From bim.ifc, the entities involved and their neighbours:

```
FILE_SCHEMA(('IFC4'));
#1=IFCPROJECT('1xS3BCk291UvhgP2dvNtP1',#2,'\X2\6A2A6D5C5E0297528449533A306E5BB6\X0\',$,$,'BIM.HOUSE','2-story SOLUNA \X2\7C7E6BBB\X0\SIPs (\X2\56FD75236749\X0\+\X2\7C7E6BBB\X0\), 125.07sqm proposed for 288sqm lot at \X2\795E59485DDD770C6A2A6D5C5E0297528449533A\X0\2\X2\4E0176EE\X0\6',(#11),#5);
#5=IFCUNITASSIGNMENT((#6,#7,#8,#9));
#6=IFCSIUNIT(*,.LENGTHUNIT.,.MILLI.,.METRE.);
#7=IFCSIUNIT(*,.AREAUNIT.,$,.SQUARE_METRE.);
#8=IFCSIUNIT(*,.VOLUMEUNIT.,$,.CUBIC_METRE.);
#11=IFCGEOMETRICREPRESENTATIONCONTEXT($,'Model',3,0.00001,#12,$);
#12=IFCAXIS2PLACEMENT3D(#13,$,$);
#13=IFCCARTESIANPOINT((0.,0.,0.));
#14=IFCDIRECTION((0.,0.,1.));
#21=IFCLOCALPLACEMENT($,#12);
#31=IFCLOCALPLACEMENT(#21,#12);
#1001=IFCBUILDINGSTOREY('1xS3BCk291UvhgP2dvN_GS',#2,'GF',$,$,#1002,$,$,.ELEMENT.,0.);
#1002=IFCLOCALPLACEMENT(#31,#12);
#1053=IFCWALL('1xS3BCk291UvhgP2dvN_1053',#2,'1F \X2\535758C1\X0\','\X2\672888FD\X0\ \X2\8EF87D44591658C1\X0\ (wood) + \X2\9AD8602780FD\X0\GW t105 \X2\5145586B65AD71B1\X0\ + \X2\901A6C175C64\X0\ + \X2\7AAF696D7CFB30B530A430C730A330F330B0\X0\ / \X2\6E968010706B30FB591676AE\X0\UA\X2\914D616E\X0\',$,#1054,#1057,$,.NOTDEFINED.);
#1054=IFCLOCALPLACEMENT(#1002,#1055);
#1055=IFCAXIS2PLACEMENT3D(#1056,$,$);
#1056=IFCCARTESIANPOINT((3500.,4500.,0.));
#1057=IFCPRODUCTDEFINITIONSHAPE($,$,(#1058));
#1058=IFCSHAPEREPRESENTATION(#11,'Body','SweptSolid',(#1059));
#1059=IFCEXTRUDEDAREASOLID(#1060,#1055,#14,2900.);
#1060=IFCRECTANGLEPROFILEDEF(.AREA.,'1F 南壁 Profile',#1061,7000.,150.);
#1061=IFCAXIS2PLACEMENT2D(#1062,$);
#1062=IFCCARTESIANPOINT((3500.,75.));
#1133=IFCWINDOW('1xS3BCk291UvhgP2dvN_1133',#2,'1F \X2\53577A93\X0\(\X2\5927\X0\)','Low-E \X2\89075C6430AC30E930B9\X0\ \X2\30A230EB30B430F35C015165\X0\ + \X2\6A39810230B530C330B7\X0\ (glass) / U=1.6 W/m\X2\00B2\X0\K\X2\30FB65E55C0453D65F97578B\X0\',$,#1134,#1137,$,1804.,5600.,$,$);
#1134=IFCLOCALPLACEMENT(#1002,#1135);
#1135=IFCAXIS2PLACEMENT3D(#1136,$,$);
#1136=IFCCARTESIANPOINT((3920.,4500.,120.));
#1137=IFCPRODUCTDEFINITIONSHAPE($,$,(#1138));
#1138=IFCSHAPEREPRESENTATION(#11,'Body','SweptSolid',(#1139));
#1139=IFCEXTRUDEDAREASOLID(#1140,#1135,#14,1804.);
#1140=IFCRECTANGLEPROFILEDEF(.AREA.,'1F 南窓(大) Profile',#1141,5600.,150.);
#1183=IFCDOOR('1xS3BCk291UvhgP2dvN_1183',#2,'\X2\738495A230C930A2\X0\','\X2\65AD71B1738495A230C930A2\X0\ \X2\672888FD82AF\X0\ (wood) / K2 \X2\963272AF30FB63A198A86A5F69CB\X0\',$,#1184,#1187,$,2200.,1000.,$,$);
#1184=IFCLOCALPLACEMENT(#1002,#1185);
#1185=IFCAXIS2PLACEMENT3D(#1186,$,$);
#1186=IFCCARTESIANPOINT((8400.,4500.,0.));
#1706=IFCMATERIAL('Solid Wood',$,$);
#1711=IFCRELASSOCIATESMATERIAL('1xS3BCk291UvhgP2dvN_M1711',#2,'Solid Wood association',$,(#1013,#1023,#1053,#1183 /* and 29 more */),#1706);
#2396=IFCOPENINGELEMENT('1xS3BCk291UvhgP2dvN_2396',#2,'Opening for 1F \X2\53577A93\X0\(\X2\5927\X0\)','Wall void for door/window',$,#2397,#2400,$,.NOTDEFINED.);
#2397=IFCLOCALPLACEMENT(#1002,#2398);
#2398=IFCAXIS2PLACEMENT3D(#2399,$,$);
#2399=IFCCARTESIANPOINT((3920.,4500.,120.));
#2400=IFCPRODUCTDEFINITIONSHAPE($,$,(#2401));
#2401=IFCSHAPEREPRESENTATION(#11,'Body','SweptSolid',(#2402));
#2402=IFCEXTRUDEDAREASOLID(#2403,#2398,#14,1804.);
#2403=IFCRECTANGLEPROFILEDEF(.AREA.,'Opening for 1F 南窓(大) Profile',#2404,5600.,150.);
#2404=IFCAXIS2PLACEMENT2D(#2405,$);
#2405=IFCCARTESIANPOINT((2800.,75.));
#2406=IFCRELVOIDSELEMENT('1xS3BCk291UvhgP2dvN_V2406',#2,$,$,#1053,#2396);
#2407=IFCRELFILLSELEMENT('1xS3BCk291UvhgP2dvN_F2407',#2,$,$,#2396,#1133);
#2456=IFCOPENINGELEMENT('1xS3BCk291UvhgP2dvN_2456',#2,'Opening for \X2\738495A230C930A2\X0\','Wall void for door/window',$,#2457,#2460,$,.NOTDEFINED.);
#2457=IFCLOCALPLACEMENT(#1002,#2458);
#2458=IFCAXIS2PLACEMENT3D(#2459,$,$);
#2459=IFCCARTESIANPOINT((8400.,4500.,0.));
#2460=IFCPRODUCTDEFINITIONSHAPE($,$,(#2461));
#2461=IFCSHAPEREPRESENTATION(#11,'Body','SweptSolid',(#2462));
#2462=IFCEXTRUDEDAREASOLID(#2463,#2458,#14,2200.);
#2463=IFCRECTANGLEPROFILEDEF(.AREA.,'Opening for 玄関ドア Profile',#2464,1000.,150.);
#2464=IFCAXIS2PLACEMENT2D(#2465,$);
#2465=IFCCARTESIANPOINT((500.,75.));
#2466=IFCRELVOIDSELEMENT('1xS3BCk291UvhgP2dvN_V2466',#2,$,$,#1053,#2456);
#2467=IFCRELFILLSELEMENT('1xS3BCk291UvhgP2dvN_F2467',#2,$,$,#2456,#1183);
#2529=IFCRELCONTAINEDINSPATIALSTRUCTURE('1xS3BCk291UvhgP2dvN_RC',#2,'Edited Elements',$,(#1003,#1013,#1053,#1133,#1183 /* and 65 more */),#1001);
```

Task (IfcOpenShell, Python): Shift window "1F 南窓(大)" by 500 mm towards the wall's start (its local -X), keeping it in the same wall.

```python
import ifcopenshell
import ifcopenshell.api.geometry
import ifcopenshell.util.placement
import ifcopenshell.util.unit

model = ifcopenshell.open("bim.ifc")
unit_scale = ifcopenshell.util.unit.calculate_unit_scale(model)

window = model.by_id(1133)
opening = window.FillsVoids[0].RelatingOpeningElement
wall = opening.VoidsElements[0].RelatingBuildingElement

wall_matrix = ifcopenshell.util.placement.get_local_placement(wall.ObjectPlacement)
shift = wall_matrix[:3, 0] * -0.5 / unit_scale
before = ifcopenshell.util.placement.get_local_placement(window.ObjectPlacement)[:3, 3].copy()

# The window is not placed relative to its opening, so move both.
for product in (opening, window):
    matrix = ifcopenshell.util.placement.get_local_placement(product.ObjectPlacement)
    matrix[:3, 3] += shift
    ifcopenshell.api.geometry.edit_object_placement(model, product=product, matrix=matrix, is_si=False)

after = ifcopenshell.util.placement.get_local_placement(window.ObjectPlacement)[:3, 3]
print("window moved by", (after - before).round(3) + 0.0)

model.write("bim-out.ifc")
```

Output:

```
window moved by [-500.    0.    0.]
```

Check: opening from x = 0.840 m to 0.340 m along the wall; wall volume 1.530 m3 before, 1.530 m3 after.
